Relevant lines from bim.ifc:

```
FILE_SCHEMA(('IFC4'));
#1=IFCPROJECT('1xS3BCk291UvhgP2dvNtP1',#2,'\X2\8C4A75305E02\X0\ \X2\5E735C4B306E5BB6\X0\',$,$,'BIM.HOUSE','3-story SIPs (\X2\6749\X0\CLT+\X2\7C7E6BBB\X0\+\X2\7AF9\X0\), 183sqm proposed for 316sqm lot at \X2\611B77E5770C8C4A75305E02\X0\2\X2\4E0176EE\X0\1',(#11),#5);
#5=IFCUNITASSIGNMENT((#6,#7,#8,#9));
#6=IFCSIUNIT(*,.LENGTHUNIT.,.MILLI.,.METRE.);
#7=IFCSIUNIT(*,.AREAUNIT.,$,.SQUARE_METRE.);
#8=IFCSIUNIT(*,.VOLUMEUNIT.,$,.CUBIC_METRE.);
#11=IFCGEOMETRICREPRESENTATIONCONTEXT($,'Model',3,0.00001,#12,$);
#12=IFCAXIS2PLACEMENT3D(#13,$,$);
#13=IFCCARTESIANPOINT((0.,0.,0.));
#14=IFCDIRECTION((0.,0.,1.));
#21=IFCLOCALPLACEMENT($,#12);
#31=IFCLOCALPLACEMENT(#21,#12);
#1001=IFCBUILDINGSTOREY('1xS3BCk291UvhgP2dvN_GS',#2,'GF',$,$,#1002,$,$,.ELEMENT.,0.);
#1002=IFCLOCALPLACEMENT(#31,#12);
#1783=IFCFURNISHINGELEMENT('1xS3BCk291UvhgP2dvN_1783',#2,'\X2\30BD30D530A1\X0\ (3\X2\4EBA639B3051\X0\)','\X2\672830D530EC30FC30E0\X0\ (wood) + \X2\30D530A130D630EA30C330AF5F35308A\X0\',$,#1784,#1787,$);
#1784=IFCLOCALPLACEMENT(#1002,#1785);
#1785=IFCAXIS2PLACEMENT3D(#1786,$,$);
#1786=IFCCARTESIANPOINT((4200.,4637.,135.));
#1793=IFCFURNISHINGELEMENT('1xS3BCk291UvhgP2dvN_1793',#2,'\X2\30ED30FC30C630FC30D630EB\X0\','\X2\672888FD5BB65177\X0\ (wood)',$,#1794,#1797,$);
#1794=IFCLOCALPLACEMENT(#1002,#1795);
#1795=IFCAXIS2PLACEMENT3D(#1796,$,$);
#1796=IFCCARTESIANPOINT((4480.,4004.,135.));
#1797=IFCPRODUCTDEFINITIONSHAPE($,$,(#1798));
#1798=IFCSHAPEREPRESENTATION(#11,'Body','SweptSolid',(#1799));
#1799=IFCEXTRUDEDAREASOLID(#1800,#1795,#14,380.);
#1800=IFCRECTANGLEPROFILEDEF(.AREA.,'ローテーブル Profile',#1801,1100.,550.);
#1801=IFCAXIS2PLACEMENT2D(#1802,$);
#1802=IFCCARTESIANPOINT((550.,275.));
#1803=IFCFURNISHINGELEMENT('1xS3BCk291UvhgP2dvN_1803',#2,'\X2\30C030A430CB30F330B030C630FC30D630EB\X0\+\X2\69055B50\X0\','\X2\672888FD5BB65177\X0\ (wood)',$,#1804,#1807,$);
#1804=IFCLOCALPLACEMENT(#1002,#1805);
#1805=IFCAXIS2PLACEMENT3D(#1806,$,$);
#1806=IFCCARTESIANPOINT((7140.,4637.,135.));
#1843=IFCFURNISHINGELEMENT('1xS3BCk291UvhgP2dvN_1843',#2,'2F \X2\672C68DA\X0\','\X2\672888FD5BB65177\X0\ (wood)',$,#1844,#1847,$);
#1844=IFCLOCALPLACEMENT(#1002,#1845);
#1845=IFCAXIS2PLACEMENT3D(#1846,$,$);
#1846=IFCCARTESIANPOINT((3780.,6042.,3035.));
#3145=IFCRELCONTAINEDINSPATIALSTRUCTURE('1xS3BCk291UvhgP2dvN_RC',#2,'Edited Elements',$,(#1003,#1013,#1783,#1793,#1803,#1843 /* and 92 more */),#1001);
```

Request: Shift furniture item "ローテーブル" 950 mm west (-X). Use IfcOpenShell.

```python
import ifcopenshell
import ifcopenshell.api.geometry
import ifcopenshell.util.placement
import ifcopenshell.util.unit

model = ifcopenshell.open("bim.ifc")
unit_scale = ifcopenshell.util.unit.calculate_unit_scale(model)

item = model.by_guid("1xS3BCk291UvhgP2dvN_1793")
matrix = ifcopenshell.util.placement.get_local_placement(item.ObjectPlacement)
matrix[0, 3] -= 0.95 / unit_scale
ifcopenshell.api.geometry.edit_object_placement(model, product=item, matrix=matrix, is_si=False)

print(ifcopenshell.util.placement.get_local_placement(item.ObjectPlacement).round(3) + 0.0)

model.write("bim_edited.ifc")
```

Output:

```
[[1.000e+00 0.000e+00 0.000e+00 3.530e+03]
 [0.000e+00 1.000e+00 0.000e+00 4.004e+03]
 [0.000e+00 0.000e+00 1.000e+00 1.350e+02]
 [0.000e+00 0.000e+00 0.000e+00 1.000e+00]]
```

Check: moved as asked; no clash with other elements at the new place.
